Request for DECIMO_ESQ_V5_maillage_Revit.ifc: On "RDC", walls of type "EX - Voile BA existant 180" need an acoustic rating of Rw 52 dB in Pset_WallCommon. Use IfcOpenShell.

First a look at what the model holds.

```python
import ifcopenshell
import ifcopenshell.util.element

model = ifcopenshell.open("DECIMO_ESQ_V5_maillage_Revit.ifc")
print(model.schema)
storey = next(s for s in model.by_type("IfcBuildingStorey") if s.Name == "RDC")
walls = [e for e in ifcopenshell.util.element.get_decomposition(storey) if e.is_a("IfcWall")]
seen = {}
for e in walls:
    element_type = ifcopenshell.util.element.get_type(e)
    key = (element_type.Name if element_type != e and element_type else None, ifcopenshell.util.element.get_pset(e, "Pset_WallCommon", "AcousticRating"))
    seen[key] = seen.get(key, 0) + 1
for (name, value), count in sorted(seen.items(), key=str):
    print(count, "x", name, "|", value)
```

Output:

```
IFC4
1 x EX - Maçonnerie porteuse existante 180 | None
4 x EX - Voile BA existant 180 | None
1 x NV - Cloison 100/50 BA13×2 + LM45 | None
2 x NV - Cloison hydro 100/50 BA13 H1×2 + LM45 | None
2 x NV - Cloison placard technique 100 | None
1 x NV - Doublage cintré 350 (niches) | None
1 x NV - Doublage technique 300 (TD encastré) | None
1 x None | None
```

```python
import ifcopenshell
import ifcopenshell.api.pset
import ifcopenshell.util.element

model = ifcopenshell.open("DECIMO_ESQ_V5_maillage_Revit.ifc")

storey = next(s for s in model.by_type("IfcBuildingStorey") if s.Name == "RDC")
walls = [e for e in ifcopenshell.util.element.get_decomposition(storey) if e.is_a("IfcWall")]

count = 0
for e in walls:
    element_type = ifcopenshell.util.element.get_type(e)
    if element_type in (None, e) or element_type.Name != "EX - Voile BA existant 180":
        continue
    # add_pset returns the element's existing set when there is one.
    pset = ifcopenshell.api.pset.add_pset(model, product=e, name="Pset_WallCommon")
    ifcopenshell.api.pset.edit_pset(model, pset=pset, properties={"AcousticRating": "Rw 52 dB"})
    count += 1

print(count, "walls updated")

model.write("DECIMO_ESQ_V5_maillage_Revit_updated.ifc")
```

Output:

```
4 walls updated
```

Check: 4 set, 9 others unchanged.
